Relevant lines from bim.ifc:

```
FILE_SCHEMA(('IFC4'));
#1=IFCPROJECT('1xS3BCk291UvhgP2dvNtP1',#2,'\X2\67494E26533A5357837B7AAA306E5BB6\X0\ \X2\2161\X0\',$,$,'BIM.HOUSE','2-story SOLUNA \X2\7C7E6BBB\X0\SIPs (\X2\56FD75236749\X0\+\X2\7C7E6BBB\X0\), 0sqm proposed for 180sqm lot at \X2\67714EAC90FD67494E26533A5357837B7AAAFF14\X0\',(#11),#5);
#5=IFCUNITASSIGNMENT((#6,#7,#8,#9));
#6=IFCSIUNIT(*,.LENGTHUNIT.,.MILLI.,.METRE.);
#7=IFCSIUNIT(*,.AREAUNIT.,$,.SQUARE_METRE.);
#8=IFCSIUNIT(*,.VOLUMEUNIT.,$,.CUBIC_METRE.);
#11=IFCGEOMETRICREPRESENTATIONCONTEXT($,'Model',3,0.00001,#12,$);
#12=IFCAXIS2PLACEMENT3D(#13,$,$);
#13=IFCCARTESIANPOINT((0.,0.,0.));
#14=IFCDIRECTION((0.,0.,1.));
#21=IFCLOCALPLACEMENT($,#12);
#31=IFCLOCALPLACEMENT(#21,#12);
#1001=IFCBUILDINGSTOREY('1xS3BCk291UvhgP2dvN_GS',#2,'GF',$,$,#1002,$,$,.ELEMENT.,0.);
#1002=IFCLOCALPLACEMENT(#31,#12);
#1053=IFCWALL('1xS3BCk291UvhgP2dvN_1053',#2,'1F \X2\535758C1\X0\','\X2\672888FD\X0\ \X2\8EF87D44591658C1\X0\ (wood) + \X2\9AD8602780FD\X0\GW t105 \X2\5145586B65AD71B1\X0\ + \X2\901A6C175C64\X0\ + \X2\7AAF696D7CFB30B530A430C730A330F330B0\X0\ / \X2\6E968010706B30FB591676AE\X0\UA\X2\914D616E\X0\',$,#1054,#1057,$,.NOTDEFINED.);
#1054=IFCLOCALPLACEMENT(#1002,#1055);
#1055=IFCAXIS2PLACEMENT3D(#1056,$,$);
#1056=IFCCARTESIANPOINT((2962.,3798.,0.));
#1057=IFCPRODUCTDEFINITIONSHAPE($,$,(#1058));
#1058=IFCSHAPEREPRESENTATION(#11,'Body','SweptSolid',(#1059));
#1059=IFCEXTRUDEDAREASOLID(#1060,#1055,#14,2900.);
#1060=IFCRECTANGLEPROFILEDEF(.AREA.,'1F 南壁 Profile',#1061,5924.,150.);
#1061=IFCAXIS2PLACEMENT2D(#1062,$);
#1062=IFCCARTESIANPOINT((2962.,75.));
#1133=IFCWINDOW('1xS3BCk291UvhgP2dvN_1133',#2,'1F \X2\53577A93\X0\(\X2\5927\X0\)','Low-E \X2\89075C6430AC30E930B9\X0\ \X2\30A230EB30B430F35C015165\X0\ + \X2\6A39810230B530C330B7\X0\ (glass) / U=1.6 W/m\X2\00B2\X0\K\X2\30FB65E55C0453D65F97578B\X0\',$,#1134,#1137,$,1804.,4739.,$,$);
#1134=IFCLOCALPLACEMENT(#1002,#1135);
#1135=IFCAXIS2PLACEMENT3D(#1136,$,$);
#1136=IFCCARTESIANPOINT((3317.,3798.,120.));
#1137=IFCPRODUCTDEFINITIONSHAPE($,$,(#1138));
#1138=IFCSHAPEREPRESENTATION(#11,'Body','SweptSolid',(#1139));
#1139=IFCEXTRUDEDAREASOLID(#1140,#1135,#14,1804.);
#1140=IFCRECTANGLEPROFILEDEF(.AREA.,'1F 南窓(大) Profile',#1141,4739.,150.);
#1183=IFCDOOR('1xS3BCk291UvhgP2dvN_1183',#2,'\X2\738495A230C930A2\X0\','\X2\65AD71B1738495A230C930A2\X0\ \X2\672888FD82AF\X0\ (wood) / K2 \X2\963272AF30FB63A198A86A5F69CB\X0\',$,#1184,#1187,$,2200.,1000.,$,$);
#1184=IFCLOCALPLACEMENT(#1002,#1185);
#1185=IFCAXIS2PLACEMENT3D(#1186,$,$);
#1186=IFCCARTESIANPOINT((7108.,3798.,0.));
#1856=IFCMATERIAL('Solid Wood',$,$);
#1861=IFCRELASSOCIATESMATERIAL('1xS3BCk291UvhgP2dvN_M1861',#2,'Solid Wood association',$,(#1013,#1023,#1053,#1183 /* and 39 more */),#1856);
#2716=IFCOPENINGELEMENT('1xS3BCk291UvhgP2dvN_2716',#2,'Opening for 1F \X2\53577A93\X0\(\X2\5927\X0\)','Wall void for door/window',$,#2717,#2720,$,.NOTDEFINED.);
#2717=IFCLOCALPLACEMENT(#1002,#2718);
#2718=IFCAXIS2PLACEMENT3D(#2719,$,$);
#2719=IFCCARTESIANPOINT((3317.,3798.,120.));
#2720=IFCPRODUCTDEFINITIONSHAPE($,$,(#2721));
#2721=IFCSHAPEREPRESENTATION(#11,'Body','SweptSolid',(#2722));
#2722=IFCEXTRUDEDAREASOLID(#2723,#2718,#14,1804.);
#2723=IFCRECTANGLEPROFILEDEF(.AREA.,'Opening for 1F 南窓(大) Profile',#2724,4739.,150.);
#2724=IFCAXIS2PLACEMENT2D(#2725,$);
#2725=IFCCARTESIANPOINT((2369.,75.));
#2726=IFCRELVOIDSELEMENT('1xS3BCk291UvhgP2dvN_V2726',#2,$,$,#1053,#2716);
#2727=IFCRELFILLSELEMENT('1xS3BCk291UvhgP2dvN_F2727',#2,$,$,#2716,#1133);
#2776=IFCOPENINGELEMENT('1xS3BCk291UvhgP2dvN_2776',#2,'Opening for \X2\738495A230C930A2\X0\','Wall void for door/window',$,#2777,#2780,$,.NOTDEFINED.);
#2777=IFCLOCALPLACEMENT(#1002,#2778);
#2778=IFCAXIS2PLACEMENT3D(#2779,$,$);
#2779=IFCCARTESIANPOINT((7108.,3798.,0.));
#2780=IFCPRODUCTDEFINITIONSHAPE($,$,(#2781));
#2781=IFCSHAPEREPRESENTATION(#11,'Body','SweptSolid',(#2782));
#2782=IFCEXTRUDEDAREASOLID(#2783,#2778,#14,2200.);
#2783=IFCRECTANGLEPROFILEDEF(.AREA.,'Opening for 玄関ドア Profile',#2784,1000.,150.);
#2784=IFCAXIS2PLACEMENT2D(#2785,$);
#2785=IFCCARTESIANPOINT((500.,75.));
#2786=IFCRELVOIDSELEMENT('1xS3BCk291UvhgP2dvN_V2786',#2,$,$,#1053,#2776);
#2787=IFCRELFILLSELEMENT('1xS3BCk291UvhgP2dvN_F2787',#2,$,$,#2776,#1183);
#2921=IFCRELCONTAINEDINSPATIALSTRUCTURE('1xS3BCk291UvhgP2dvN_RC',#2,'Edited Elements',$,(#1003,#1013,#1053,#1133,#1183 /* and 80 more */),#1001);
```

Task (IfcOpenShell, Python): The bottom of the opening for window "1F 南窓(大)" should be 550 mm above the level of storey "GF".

```python
import numpy as np
import ifcopenshell
import ifcopenshell.api.geometry
import ifcopenshell.geom
import ifcopenshell.util.element
import ifcopenshell.util.placement
import ifcopenshell.util.shape
import ifcopenshell.util.unit

model = ifcopenshell.open("bim.ifc")
unit_scale = ifcopenshell.util.unit.calculate_unit_scale(model)

window = model.by_guid("1xS3BCk291UvhgP2dvN_1133")
opening = window.FillsVoids[0].RelatingOpeningElement
storey = ifcopenshell.util.element.get_container(window, ifc_class="IfcBuildingStorey")
level = ifcopenshell.util.placement.get_local_placement(storey.ObjectPlacement)[2, 3]

# The opening's origin need not be at the sill, so measure its lowest point.
shape = ifcopenshell.geom.create_shape(ifcopenshell.geom.settings(), opening)
bottom = ifcopenshell.util.shape.get_shape_bottom_elevation(shape, shape.geometry) / unit_scale
dz = level + 0.55 / unit_scale - bottom

shift = np.array([0.0, 0.0, dz])
# The window is not placed relative to its opening, so move both.
for product in (opening, window):
    matrix = ifcopenshell.util.placement.get_local_placement(product.ObjectPlacement)
    matrix[:3, 3] += shift
    ifcopenshell.api.geometry.edit_object_placement(model, product=product, matrix=matrix, is_si=False)

print(f"moved by {dz * unit_scale:+.3f} m")

model.write("bim_v2.ifc")
```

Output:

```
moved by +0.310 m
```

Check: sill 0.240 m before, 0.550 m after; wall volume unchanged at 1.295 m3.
